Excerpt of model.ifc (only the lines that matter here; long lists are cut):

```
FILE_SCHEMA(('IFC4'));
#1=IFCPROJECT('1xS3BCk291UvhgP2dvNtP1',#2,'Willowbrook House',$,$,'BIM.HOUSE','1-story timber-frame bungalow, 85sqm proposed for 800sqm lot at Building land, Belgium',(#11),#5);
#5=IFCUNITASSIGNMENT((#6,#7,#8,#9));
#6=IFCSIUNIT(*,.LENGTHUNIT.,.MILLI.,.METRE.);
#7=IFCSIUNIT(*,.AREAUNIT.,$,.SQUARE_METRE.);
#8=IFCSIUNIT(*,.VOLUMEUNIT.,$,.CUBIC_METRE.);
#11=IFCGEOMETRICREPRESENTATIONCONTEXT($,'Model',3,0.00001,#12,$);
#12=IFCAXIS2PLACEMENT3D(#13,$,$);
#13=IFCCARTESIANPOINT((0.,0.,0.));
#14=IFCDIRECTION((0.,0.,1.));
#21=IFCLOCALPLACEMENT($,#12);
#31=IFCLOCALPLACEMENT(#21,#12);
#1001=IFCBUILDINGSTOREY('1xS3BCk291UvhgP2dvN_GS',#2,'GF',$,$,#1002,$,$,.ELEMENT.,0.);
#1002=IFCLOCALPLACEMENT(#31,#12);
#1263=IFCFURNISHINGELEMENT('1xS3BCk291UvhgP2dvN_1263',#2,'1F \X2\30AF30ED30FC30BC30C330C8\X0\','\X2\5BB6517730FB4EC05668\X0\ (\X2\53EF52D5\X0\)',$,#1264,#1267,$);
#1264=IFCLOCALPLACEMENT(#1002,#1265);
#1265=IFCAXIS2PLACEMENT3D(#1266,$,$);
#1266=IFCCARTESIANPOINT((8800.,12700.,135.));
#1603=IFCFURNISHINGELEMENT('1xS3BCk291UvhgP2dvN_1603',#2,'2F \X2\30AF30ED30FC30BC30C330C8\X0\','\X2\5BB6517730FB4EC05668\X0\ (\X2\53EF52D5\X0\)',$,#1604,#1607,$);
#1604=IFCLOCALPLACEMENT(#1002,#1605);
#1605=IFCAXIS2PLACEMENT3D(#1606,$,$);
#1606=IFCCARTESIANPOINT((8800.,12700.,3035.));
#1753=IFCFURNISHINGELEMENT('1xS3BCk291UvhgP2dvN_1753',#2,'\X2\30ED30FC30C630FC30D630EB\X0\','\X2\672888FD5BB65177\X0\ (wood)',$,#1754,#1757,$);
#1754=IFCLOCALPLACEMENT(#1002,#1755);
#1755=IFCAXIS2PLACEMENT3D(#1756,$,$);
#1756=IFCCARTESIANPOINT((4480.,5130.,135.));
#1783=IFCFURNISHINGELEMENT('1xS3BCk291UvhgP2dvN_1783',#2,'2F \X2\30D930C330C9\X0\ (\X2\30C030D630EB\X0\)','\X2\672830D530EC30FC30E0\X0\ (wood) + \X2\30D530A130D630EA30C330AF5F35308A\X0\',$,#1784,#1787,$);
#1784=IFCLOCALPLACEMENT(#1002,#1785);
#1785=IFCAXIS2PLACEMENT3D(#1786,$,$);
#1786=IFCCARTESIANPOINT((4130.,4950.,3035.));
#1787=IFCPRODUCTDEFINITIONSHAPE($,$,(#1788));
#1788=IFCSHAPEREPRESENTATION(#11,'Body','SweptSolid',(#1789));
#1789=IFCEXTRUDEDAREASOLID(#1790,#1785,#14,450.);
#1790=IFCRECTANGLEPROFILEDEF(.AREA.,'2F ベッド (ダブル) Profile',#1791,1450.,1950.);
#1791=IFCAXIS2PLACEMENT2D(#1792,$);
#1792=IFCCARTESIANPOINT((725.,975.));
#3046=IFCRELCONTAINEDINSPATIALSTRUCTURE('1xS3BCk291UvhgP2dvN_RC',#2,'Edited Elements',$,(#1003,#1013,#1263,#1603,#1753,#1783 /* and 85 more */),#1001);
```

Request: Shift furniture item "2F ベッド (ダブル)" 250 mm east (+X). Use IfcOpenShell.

```python
import ifcopenshell
import ifcopenshell.api.geometry
import ifcopenshell.util.placement

model = ifcopenshell.open("model.ifc")

item = model.by_guid("1xS3BCk291UvhgP2dvN_1783")
matrix = ifcopenshell.util.placement.get_local_placement(item.ObjectPlacement)
matrix[0, 3] += 250.0
ifcopenshell.api.geometry.edit_object_placement(model, product=item, matrix=matrix, is_si=False)

print(ifcopenshell.util.placement.get_local_placement(item.ObjectPlacement).round(3) + 0.0)

model.write("model_edited.ifc")
```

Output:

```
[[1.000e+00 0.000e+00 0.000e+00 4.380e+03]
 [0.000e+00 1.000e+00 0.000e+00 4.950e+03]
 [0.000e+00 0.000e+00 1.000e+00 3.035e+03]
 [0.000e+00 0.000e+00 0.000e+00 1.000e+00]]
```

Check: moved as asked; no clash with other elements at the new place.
